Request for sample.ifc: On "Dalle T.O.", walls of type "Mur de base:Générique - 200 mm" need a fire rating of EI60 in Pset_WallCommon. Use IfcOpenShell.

First a look at what the model holds.

```python
import ifcopenshell
import ifcopenshell.util.element

model = ifcopenshell.open("sample.ifc")
print(model.schema)
storey = next(s for s in model.by_type("IfcBuildingStorey") if s.Name == "Dalle T.O.")
walls = [e for e in ifcopenshell.util.element.get_decomposition(storey) if e.is_a("IfcWall")]
seen = {}
for e in walls:
    element_type = ifcopenshell.util.element.get_type(e)
    key = (element_type.Name if element_type != e and element_type else None, ifcopenshell.util.element.get_pset(e, "Pset_WallCommon", "FireRating"))
    seen[key] = seen.get(key, 0) + 1
for (name, value), count in sorted(seen.items(), key=str):
    print(count, "x", name, "|", value)
```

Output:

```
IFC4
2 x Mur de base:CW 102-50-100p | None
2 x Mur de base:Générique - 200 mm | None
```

```python
import ifcopenshell
import ifcopenshell.api.pset
import ifcopenshell.util.element

model = ifcopenshell.open("sample.ifc")

storey = next(s for s in model.by_type("IfcBuildingStorey") if s.Name == "Dalle T.O.")
walls = [e for e in ifcopenshell.util.element.get_decomposition(storey) if e.is_a("IfcWall")]

count = 0
for e in walls:
    element_type = ifcopenshell.util.element.get_type(e)
    if element_type in (None, e) or element_type.Name != "Mur de base:Générique - 200 mm":
        continue
    # add_pset returns the element's existing set when there is one.
    pset = ifcopenshell.api.pset.add_pset(model, product=e, name="Pset_WallCommon")
    ifcopenshell.api.pset.edit_pset(model, pset=pset, properties={"FireRating": "EI60"})
    count += 1

print(count, "walls updated")

model.write("sample_rev.ifc")
```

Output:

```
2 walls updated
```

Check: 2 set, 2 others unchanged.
